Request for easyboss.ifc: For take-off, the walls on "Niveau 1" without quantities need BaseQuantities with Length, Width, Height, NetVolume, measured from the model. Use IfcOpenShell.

First a look at what the model holds.

```python
import ifcopenshell
import ifcopenshell.util.element
import ifcopenshell.util.unit

model = ifcopenshell.open("easyboss.ifc")
print(model.schema)
for unit_type in ("LENGTHUNIT", "AREAUNIT", "VOLUMEUNIT"):
    print(unit_type, ifcopenshell.util.unit.calculate_unit_scale(model, unit_type))
storey = next(s for s in model.by_type("IfcBuildingStorey") if s.Name == "Niveau 1")
walls = [e for e in ifcopenshell.util.element.get_decomposition(storey) if e.is_a("IfcWall")]
for e in sorted(walls, key=lambda e: e.id()):
    print(e.id(), e.is_a(), e.Name, list(ifcopenshell.util.element.get_psets(e, qtos_only=True)), sep=" | ")
```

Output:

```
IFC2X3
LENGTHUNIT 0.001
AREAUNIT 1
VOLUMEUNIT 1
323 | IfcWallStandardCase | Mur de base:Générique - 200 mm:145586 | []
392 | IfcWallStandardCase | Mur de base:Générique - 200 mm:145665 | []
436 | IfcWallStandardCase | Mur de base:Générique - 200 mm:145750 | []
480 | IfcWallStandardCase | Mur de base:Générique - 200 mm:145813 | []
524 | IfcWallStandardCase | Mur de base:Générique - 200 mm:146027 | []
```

```python
import ifcopenshell
import ifcopenshell.api.pset
import ifcopenshell.geom
import ifcopenshell.util.element
import ifcopenshell.util.shape
import ifcopenshell.util.unit

model = ifcopenshell.open("easyboss.ifc")
unit_scale = ifcopenshell.util.unit.calculate_unit_scale(model)
volume_scale = ifcopenshell.util.unit.calculate_unit_scale(model, "VOLUMEUNIT")
settings = ifcopenshell.geom.settings()

storey = next(s for s in model.by_type("IfcBuildingStorey") if s.Name == "Niveau 1")
walls = [e for e in ifcopenshell.util.element.get_decomposition(storey) if e.is_a("IfcWall")]

for e in sorted(walls, key=lambda e: e.id()):
    if ifcopenshell.util.element.get_psets(e, qtos_only=True, should_inherit=False):
        continue
    # Geometry comes back in metres, in the element's own axes.
    shape = ifcopenshell.geom.create_shape(settings, e)
    values = {
        "Length": ifcopenshell.util.shape.get_x(shape.geometry) / unit_scale,
        "Width": ifcopenshell.util.shape.get_y(shape.geometry) / unit_scale,
        "Height": ifcopenshell.util.shape.get_z(shape.geometry) / unit_scale,
        "NetVolume": ifcopenshell.util.shape.get_volume(shape.geometry) / volume_scale,
    }
    qto = ifcopenshell.api.pset.add_qto(model, product=e, name="BaseQuantities")
    ifcopenshell.api.pset.edit_qto(model, qto=qto, properties=values)
    print(e.id(), {k: round(v, 3) for k, v in values.items()})

model.write("easyboss_rev.ifc")
```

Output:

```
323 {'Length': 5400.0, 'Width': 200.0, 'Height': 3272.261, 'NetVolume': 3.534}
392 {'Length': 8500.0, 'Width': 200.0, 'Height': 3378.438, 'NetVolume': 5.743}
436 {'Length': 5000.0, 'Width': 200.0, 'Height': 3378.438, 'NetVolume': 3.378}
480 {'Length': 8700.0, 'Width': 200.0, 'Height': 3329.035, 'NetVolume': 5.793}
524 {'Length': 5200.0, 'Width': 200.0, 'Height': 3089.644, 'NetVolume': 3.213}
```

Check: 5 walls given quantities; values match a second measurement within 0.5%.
